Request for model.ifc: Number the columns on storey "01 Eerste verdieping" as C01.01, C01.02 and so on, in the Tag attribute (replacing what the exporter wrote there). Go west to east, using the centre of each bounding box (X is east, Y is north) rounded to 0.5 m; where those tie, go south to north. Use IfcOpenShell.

First a look at what the model holds.

```python
import ifcopenshell
import ifcopenshell.util.element
import ifcopenshell.util.placement

model = ifcopenshell.open("model.ifc")
print(model.schema)
storey = next(s for s in model.by_type("IfcBuildingStorey") if s.Name == "01 Eerste verdieping")
columns = [e for e in ifcopenshell.util.element.get_decomposition(storey) if e.is_a("IfcColumn")]
for e in sorted(columns, key=lambda e: e.id()):
    origin = ifcopenshell.util.placement.get_local_placement(e.ObjectPlacement)[:3, 3]
    print(e.id(), e.Tag, e.Name, origin.round(2) + 0.0, sep=" | ")
```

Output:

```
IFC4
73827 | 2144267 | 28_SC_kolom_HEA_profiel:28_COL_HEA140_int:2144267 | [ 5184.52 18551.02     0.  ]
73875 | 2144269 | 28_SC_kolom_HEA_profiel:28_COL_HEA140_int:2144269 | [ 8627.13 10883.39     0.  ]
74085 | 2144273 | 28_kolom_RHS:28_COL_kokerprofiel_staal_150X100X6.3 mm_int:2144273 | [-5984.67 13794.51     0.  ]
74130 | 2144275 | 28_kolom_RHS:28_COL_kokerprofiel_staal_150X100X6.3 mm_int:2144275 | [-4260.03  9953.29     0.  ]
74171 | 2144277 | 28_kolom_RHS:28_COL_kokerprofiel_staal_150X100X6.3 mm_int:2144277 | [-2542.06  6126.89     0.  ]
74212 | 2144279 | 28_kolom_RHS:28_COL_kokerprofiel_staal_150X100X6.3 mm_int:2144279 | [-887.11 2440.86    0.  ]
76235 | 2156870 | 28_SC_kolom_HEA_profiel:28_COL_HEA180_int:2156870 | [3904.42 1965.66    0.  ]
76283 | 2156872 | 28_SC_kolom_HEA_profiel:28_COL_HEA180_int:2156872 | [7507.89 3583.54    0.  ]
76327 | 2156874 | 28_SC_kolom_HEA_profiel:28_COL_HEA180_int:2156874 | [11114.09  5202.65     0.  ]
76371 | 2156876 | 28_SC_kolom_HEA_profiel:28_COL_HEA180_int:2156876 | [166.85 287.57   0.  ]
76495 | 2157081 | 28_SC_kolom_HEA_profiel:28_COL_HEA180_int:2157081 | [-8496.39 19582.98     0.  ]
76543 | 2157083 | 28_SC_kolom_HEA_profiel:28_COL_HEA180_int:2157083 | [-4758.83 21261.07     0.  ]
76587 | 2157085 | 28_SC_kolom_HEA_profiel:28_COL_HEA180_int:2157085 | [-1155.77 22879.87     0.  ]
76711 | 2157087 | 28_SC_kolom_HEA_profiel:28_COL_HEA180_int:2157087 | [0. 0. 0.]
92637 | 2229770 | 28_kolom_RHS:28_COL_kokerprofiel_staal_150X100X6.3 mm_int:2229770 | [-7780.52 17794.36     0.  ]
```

```python
import ifcopenshell
import ifcopenshell.geom
import ifcopenshell.util.element
import ifcopenshell.util.shape

model = ifcopenshell.open("model.ifc")
settings = ifcopenshell.geom.settings()
settings.set("use-world-coords", True)


def centre(element):
    shape = ifcopenshell.geom.create_shape(settings, element)
    return ifcopenshell.util.shape.get_bbox_centroid(shape.geometry)


storey = next(s for s in model.by_type("IfcBuildingStorey") if s.Name == "01 Eerste verdieping")
columns = [e for e in ifcopenshell.util.element.get_decomposition(storey) if e.is_a("IfcColumn")]

# Insertion points can sit at a corner or the storey origin, so sort by the geometry (in metres).
centres = {e: centre(e) for e in columns}
columns.sort(key=lambda e: (round(centres[e][0] / 0.5), centres[e][1]))

for i, e in enumerate(columns, start=1):
    number = f"C01.{i:02d}"
    e.Tag = number
    print(e.id(), number)

model.write("model_rev.ifc")
```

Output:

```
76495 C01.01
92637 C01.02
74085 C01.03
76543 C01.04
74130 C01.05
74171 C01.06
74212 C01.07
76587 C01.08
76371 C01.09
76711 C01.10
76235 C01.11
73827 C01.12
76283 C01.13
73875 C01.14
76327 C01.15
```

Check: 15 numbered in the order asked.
